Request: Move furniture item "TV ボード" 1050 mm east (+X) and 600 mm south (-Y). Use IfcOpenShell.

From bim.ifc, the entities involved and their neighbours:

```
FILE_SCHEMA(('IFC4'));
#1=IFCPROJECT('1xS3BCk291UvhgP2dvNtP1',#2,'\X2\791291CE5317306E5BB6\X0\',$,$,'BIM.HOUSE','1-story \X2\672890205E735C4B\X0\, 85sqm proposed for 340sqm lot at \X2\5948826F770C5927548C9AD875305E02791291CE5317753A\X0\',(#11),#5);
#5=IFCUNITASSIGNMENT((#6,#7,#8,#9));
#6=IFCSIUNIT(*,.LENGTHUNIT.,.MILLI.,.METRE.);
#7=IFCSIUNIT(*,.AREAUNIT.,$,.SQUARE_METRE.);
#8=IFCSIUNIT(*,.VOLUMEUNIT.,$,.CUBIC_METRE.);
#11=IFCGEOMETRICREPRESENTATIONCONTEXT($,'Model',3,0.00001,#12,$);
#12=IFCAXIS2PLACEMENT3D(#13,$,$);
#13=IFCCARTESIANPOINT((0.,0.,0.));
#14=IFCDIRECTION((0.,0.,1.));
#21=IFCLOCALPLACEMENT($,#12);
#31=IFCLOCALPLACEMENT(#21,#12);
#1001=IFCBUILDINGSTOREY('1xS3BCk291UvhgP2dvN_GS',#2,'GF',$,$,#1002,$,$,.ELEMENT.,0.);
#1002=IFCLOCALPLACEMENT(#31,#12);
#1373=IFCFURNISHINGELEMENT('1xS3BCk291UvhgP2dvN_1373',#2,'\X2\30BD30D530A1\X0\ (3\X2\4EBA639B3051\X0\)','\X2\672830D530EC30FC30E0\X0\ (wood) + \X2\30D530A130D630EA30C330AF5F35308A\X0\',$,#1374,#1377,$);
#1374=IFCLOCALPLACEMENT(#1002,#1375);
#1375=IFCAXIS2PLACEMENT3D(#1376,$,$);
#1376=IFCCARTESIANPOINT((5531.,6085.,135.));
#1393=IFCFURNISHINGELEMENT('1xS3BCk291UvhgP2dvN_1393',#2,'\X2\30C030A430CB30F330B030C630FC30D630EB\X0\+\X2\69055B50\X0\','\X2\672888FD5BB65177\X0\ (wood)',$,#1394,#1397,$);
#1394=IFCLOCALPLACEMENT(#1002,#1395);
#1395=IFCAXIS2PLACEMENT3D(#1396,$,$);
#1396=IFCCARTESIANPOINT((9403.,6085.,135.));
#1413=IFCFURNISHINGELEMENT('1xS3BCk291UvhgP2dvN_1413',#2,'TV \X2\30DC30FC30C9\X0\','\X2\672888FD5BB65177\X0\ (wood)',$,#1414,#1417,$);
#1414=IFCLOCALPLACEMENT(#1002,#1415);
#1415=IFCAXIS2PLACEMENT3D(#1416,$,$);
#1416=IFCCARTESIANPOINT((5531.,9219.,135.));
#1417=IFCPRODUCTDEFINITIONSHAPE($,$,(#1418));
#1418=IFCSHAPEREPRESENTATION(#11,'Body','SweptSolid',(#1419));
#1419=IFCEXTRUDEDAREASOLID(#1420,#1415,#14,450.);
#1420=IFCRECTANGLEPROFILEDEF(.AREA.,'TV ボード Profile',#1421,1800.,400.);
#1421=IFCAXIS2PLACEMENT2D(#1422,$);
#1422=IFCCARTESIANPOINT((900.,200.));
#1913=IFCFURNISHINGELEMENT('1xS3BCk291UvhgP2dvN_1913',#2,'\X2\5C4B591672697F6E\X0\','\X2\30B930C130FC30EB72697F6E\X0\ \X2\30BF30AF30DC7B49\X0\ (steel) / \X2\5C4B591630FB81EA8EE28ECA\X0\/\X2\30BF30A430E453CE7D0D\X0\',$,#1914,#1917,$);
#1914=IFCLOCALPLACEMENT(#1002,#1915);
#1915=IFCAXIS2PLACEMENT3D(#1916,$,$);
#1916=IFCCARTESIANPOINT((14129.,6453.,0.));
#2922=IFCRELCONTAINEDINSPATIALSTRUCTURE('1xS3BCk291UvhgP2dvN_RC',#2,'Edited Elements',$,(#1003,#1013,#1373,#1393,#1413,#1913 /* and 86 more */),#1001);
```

```python
import ifcopenshell
import ifcopenshell.api.geometry
import ifcopenshell.util.placement

model = ifcopenshell.open("bim.ifc")

item = model.by_guid("1xS3BCk291UvhgP2dvN_1413")
matrix = ifcopenshell.util.placement.get_local_placement(item.ObjectPlacement)
matrix[0, 3] += 1050.0
matrix[1, 3] -= 600.0
ifcopenshell.api.geometry.edit_object_placement(model, product=item, matrix=matrix, is_si=False)

print(ifcopenshell.util.placement.get_local_placement(item.ObjectPlacement).round(3) + 0.0)

model.write("bim_v2.ifc")
```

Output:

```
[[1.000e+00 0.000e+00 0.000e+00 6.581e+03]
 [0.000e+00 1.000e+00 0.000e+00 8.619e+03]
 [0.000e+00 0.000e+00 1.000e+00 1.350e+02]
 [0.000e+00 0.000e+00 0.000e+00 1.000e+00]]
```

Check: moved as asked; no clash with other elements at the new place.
